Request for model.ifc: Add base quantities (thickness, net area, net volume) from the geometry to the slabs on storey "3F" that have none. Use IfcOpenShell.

First a look at what the model holds.

```python
import ifcopenshell
import ifcopenshell.util.element
import ifcopenshell.util.unit

model = ifcopenshell.open("model.ifc")
print(model.schema)
for unit_type in ("LENGTHUNIT", "AREAUNIT", "VOLUMEUNIT"):
    print(unit_type, ifcopenshell.util.unit.calculate_unit_scale(model, unit_type))
storey = next(s for s in model.by_type("IfcBuildingStorey") if s.Name == "3F")
slabs = [e for e in ifcopenshell.util.element.get_decomposition(storey) if e.is_a("IfcSlab")]
for e in sorted(slabs, key=lambda e: e.id()):
    print(e.id(), e.is_a(), e.Name, list(ifcopenshell.util.element.get_psets(e, qtos_only=True)), sep=" | ")
```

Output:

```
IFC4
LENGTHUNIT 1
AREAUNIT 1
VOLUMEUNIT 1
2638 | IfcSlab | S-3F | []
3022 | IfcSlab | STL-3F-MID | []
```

```python
import ifcopenshell
import ifcopenshell.api.pset
import ifcopenshell.geom
import ifcopenshell.util.element
import ifcopenshell.util.shape
import ifcopenshell.util.unit

model = ifcopenshell.open("model.ifc")
unit_scale = ifcopenshell.util.unit.calculate_unit_scale(model)
area_scale = ifcopenshell.util.unit.calculate_unit_scale(model, "AREAUNIT")
volume_scale = ifcopenshell.util.unit.calculate_unit_scale(model, "VOLUMEUNIT")
settings = ifcopenshell.geom.settings()

storey = next(s for s in model.by_type("IfcBuildingStorey") if s.Name == "3F")
slabs = [e for e in ifcopenshell.util.element.get_decomposition(storey) if e.is_a("IfcSlab")]

for e in sorted(slabs, key=lambda e: e.id()):
    if ifcopenshell.util.element.get_psets(e, qtos_only=True, should_inherit=False):
        continue
    # Geometry comes back in metres, in the element's own axes.
    shape = ifcopenshell.geom.create_shape(settings, e)
    values = {
        "Width": ifcopenshell.util.shape.get_z(shape.geometry) / unit_scale,
        "NetArea": ifcopenshell.util.shape.get_footprint_area(shape.geometry) / area_scale,
        "NetVolume": ifcopenshell.util.shape.get_volume(shape.geometry) / volume_scale,
    }
    qto = ifcopenshell.api.pset.add_qto(model, product=e, name="Qto_SlabBaseQuantities")
    ifcopenshell.api.pset.edit_qto(model, qto=qto, properties=values)
    print(e.id(), {k: round(v, 3) for k, v in values.items()})

model.write("model_rev.ifc")
```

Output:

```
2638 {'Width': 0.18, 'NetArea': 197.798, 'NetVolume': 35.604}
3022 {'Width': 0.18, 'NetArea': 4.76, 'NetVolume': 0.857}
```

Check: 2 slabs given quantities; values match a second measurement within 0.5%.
